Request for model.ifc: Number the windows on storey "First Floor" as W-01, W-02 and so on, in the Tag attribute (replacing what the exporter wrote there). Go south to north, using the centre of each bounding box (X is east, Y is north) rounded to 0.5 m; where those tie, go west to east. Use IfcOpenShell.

First a look at what the model holds.

```python
import ifcopenshell
import ifcopenshell.util.element
import ifcopenshell.util.placement

model = ifcopenshell.open("model.ifc")
print(model.schema)
storey = next(s for s in model.by_type("IfcBuildingStorey") if s.Name == "First Floor")
windows = [e for e in ifcopenshell.util.element.get_decomposition(storey) if e.is_a("IfcWindow")]
for e in sorted(windows, key=lambda e: e.id()):
    origin = ifcopenshell.util.placement.get_local_placement(e.ObjectPlacement)[:3, 3]
    print(e.id(), e.Tag, e.Name, origin.round(2) + 0.0, sep=" | ")
```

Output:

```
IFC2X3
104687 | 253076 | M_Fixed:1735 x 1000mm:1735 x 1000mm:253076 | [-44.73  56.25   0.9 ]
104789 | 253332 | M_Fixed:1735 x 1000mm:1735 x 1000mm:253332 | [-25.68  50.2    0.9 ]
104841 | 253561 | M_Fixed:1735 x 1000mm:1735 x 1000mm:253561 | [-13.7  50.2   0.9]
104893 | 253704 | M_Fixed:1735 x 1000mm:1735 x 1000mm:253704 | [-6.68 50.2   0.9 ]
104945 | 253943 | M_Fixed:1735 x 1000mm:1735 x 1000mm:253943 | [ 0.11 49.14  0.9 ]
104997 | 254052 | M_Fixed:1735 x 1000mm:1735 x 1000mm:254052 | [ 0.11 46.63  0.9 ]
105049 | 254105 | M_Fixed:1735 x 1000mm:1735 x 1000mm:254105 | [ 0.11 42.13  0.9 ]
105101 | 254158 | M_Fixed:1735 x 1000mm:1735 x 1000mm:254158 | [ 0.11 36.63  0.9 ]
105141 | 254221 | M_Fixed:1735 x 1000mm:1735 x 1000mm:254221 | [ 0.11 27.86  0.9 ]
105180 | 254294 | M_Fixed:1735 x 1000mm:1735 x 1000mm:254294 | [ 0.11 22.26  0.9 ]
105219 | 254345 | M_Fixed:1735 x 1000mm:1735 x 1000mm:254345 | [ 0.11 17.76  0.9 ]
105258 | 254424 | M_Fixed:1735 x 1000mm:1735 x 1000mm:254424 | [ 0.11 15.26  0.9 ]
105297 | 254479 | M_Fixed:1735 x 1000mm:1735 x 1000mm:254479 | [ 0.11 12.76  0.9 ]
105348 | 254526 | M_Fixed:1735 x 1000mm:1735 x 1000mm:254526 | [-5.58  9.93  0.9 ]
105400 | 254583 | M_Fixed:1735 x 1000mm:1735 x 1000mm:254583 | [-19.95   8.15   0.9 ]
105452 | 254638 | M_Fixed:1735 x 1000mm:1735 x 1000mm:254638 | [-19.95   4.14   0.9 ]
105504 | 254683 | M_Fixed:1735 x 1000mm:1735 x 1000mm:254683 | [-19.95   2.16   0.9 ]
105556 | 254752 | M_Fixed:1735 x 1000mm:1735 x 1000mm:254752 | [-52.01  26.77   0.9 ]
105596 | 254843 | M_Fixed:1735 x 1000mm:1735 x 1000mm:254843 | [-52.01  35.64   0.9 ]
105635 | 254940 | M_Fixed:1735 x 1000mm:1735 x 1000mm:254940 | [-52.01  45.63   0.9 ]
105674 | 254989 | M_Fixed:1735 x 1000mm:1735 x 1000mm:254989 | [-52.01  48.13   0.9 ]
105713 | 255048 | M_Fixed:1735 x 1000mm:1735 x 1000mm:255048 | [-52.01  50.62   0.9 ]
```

```python
import ifcopenshell
import ifcopenshell.geom
import ifcopenshell.util.element
import ifcopenshell.util.shape

model = ifcopenshell.open("model.ifc")
settings = ifcopenshell.geom.settings()
settings.set("use-world-coords", True)


def centre(element):
    shape = ifcopenshell.geom.create_shape(settings, element)
    return ifcopenshell.util.shape.get_bbox_centroid(shape.geometry)


storey = next(s for s in model.by_type("IfcBuildingStorey") if s.Name == "First Floor")
windows = [e for e in ifcopenshell.util.element.get_decomposition(storey) if e.is_a("IfcWindow")]

# Insertion points can sit at a corner or the storey origin, so sort by the geometry (in metres).
centres = {e: centre(e) for e in windows}
windows.sort(key=lambda e: (round(centres[e][1] / 0.5), centres[e][0]))

for i, e in enumerate(windows, start=1):
    number = f"W-{i:02d}"
    e.Tag = number
    print(e.id(), number)

model.write("model-out.ifc")
```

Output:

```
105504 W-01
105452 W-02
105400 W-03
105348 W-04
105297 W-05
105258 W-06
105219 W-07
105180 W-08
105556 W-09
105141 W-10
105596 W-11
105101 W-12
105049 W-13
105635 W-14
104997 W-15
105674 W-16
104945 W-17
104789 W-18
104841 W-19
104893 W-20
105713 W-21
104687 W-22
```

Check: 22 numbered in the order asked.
